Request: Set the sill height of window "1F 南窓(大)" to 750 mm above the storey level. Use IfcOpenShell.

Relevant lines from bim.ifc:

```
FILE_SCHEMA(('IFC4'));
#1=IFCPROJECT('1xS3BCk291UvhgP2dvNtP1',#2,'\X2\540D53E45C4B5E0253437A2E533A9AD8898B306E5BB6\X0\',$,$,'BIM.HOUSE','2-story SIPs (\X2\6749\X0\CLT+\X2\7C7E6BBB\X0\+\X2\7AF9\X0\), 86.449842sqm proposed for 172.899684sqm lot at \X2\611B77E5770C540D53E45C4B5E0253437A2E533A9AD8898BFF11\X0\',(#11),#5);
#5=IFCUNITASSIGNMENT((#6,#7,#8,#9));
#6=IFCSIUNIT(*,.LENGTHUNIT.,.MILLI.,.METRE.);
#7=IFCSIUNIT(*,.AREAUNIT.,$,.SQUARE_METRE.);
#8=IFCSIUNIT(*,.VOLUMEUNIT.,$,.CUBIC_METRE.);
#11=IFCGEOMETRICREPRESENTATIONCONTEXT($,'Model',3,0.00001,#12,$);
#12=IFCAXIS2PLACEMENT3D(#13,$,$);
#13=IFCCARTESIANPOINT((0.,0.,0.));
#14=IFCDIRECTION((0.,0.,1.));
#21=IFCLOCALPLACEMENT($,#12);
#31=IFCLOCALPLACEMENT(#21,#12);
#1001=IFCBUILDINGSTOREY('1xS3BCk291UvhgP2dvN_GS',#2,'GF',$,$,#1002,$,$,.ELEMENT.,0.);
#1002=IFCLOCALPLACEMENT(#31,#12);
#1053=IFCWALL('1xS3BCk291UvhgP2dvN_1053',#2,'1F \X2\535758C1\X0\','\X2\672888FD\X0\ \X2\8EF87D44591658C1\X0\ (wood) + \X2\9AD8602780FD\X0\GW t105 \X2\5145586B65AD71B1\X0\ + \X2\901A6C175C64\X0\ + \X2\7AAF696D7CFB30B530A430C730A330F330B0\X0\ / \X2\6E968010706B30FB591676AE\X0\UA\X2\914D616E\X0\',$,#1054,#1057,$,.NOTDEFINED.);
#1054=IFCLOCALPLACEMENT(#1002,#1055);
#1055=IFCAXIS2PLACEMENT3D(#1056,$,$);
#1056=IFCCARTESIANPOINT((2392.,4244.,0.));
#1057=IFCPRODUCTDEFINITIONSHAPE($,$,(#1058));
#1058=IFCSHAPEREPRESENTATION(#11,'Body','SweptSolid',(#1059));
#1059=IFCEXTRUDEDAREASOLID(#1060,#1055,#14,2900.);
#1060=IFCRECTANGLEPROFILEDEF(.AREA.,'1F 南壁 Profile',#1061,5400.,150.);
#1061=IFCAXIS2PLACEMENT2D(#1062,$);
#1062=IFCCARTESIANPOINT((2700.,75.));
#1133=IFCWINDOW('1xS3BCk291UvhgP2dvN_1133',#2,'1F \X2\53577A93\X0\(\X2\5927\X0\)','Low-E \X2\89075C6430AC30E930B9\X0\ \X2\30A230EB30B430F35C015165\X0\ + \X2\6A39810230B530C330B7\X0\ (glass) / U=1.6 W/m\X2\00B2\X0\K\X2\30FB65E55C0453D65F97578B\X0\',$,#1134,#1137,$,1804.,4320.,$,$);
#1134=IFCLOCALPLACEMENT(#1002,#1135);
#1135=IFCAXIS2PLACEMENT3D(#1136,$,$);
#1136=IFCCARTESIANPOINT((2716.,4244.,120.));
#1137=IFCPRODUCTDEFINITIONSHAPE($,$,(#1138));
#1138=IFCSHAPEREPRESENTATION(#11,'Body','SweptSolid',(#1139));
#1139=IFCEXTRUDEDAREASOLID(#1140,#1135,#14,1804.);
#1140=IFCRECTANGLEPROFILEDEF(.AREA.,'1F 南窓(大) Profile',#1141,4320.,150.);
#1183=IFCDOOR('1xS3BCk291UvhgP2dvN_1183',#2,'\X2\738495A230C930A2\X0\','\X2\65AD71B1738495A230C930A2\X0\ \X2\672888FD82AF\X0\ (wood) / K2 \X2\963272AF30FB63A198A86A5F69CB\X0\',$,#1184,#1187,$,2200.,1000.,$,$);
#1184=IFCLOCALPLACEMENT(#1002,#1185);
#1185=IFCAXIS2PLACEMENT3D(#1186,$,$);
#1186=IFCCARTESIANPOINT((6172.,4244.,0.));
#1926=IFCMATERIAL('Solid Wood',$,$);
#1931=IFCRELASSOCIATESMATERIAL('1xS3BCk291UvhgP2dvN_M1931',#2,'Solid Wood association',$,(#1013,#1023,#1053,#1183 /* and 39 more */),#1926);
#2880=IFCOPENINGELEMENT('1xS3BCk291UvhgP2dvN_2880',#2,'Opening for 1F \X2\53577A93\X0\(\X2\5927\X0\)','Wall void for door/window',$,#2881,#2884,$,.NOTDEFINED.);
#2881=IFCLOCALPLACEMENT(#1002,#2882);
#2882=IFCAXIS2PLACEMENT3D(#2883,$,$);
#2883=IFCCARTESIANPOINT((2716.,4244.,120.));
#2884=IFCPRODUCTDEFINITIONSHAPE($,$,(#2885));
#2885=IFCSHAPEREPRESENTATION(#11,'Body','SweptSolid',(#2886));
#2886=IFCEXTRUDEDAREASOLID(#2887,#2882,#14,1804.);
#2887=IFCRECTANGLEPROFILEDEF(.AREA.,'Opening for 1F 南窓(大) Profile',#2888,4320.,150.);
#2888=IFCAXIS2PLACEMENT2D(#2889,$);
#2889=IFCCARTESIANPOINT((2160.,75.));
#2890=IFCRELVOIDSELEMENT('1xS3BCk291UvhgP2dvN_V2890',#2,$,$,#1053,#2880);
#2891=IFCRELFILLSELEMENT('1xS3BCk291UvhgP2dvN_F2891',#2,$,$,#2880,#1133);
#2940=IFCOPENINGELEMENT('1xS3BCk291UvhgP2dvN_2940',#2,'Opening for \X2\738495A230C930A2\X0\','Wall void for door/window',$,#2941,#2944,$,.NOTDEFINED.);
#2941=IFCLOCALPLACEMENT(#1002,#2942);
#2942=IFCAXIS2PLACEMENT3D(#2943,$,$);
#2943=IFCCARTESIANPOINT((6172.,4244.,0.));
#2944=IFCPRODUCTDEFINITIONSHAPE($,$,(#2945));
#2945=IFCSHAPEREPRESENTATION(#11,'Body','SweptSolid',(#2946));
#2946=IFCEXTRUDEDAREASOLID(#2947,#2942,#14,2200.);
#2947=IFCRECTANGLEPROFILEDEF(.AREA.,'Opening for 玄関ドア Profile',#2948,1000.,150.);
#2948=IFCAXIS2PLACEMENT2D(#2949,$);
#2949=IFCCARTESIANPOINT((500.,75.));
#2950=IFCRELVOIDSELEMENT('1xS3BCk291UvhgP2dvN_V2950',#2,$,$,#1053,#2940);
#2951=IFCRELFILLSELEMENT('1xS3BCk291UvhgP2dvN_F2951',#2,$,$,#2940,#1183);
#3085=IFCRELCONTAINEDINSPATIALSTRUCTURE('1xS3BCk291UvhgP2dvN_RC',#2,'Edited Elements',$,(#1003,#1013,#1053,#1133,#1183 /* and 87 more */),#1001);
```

```python
import numpy as np
import ifcopenshell
import ifcopenshell.api.geometry
import ifcopenshell.geom
import ifcopenshell.util.element
import ifcopenshell.util.placement
import ifcopenshell.util.shape
import ifcopenshell.util.unit

model = ifcopenshell.open("bim.ifc")
unit_scale = ifcopenshell.util.unit.calculate_unit_scale(model)

window = model.by_guid("1xS3BCk291UvhgP2dvN_1133")
opening = window.FillsVoids[0].RelatingOpeningElement
storey = ifcopenshell.util.element.get_container(window, ifc_class="IfcBuildingStorey")
level = ifcopenshell.util.placement.get_local_placement(storey.ObjectPlacement)[2, 3]

# The opening's origin need not be at the sill, so measure its lowest point.
shape = ifcopenshell.geom.create_shape(ifcopenshell.geom.settings(), opening)
bottom = ifcopenshell.util.shape.get_shape_bottom_elevation(shape, shape.geometry) / unit_scale
dz = level + 0.75 / unit_scale - bottom

shift = np.array([0.0, 0.0, dz])
# The window is not placed relative to its opening, so move both.
for product in (opening, window):
    matrix = ifcopenshell.util.placement.get_local_placement(product.ObjectPlacement)
    matrix[:3, 3] += shift
    ifcopenshell.api.geometry.edit_object_placement(model, product=product, matrix=matrix, is_si=False)

print(f"moved by {dz * unit_scale:+.3f} m")

model.write("bim_updated.ifc")
```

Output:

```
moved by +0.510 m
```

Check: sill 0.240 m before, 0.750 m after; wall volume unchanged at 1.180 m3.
